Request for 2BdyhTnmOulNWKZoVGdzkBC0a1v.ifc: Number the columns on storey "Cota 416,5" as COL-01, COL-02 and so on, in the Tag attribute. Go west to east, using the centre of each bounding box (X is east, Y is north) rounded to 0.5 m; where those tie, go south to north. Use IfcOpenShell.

First a look at what the model holds.

```python
import ifcopenshell
import ifcopenshell.util.element
import ifcopenshell.util.placement

model = ifcopenshell.open("2BdyhTnmOulNWKZoVGdzkBC0a1v.ifc")
print(model.schema)
storey = next(s for s in model.by_type("IfcBuildingStorey") if s.Name == "Cota 416,5")
columns = [e for e in ifcopenshell.util.element.get_decomposition(storey) if e.is_a("IfcColumn")]
for e in sorted(columns, key=lambda e: e.id()):
    origin = ifcopenshell.util.placement.get_local_placement(e.ObjectPlacement)[:3, 3]
    print(e.id(), e.Tag, e.Name, origin.round(2) + 0.0, sep=" | ")
```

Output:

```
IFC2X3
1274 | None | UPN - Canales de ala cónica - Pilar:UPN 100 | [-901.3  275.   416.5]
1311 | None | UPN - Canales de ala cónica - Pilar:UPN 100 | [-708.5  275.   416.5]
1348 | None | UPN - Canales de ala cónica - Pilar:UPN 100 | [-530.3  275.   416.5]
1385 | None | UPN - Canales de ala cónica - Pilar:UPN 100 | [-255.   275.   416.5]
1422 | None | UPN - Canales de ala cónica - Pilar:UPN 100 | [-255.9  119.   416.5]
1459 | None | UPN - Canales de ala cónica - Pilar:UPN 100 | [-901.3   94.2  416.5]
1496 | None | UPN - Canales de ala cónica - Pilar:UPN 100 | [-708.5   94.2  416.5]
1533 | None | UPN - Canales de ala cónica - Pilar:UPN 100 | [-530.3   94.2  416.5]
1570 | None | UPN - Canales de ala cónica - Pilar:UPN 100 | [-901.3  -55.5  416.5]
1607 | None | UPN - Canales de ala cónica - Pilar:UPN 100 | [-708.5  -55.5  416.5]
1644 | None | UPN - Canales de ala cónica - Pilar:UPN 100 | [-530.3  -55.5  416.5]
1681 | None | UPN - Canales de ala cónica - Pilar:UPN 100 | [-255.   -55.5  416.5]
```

```python
import ifcopenshell
import ifcopenshell.geom
import ifcopenshell.util.element
import ifcopenshell.util.shape

model = ifcopenshell.open("2BdyhTnmOulNWKZoVGdzkBC0a1v.ifc")
settings = ifcopenshell.geom.settings()
settings.set("use-world-coords", True)


def centre(element):
    shape = ifcopenshell.geom.create_shape(settings, element)
    return ifcopenshell.util.shape.get_bbox_centroid(shape.geometry)


storey = next(s for s in model.by_type("IfcBuildingStorey") if s.Name == "Cota 416,5")
columns = [e for e in ifcopenshell.util.element.get_decomposition(storey) if e.is_a("IfcColumn")]

# Insertion points can sit at a corner or the storey origin, so sort by the geometry (in metres).
centres = {e: centre(e) for e in columns}
columns.sort(key=lambda e: (round(centres[e][0] / 0.5), centres[e][1]))

for i, e in enumerate(columns, start=1):
    number = f"COL-{i:02d}"
    e.Tag = number
    print(e.id(), number)

model.write("2BdyhTnmOulNWKZoVGdzkBC0a1v_rev.ifc")
```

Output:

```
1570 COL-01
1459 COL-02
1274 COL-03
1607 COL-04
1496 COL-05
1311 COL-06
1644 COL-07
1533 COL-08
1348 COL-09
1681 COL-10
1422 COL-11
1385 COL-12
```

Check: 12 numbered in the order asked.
